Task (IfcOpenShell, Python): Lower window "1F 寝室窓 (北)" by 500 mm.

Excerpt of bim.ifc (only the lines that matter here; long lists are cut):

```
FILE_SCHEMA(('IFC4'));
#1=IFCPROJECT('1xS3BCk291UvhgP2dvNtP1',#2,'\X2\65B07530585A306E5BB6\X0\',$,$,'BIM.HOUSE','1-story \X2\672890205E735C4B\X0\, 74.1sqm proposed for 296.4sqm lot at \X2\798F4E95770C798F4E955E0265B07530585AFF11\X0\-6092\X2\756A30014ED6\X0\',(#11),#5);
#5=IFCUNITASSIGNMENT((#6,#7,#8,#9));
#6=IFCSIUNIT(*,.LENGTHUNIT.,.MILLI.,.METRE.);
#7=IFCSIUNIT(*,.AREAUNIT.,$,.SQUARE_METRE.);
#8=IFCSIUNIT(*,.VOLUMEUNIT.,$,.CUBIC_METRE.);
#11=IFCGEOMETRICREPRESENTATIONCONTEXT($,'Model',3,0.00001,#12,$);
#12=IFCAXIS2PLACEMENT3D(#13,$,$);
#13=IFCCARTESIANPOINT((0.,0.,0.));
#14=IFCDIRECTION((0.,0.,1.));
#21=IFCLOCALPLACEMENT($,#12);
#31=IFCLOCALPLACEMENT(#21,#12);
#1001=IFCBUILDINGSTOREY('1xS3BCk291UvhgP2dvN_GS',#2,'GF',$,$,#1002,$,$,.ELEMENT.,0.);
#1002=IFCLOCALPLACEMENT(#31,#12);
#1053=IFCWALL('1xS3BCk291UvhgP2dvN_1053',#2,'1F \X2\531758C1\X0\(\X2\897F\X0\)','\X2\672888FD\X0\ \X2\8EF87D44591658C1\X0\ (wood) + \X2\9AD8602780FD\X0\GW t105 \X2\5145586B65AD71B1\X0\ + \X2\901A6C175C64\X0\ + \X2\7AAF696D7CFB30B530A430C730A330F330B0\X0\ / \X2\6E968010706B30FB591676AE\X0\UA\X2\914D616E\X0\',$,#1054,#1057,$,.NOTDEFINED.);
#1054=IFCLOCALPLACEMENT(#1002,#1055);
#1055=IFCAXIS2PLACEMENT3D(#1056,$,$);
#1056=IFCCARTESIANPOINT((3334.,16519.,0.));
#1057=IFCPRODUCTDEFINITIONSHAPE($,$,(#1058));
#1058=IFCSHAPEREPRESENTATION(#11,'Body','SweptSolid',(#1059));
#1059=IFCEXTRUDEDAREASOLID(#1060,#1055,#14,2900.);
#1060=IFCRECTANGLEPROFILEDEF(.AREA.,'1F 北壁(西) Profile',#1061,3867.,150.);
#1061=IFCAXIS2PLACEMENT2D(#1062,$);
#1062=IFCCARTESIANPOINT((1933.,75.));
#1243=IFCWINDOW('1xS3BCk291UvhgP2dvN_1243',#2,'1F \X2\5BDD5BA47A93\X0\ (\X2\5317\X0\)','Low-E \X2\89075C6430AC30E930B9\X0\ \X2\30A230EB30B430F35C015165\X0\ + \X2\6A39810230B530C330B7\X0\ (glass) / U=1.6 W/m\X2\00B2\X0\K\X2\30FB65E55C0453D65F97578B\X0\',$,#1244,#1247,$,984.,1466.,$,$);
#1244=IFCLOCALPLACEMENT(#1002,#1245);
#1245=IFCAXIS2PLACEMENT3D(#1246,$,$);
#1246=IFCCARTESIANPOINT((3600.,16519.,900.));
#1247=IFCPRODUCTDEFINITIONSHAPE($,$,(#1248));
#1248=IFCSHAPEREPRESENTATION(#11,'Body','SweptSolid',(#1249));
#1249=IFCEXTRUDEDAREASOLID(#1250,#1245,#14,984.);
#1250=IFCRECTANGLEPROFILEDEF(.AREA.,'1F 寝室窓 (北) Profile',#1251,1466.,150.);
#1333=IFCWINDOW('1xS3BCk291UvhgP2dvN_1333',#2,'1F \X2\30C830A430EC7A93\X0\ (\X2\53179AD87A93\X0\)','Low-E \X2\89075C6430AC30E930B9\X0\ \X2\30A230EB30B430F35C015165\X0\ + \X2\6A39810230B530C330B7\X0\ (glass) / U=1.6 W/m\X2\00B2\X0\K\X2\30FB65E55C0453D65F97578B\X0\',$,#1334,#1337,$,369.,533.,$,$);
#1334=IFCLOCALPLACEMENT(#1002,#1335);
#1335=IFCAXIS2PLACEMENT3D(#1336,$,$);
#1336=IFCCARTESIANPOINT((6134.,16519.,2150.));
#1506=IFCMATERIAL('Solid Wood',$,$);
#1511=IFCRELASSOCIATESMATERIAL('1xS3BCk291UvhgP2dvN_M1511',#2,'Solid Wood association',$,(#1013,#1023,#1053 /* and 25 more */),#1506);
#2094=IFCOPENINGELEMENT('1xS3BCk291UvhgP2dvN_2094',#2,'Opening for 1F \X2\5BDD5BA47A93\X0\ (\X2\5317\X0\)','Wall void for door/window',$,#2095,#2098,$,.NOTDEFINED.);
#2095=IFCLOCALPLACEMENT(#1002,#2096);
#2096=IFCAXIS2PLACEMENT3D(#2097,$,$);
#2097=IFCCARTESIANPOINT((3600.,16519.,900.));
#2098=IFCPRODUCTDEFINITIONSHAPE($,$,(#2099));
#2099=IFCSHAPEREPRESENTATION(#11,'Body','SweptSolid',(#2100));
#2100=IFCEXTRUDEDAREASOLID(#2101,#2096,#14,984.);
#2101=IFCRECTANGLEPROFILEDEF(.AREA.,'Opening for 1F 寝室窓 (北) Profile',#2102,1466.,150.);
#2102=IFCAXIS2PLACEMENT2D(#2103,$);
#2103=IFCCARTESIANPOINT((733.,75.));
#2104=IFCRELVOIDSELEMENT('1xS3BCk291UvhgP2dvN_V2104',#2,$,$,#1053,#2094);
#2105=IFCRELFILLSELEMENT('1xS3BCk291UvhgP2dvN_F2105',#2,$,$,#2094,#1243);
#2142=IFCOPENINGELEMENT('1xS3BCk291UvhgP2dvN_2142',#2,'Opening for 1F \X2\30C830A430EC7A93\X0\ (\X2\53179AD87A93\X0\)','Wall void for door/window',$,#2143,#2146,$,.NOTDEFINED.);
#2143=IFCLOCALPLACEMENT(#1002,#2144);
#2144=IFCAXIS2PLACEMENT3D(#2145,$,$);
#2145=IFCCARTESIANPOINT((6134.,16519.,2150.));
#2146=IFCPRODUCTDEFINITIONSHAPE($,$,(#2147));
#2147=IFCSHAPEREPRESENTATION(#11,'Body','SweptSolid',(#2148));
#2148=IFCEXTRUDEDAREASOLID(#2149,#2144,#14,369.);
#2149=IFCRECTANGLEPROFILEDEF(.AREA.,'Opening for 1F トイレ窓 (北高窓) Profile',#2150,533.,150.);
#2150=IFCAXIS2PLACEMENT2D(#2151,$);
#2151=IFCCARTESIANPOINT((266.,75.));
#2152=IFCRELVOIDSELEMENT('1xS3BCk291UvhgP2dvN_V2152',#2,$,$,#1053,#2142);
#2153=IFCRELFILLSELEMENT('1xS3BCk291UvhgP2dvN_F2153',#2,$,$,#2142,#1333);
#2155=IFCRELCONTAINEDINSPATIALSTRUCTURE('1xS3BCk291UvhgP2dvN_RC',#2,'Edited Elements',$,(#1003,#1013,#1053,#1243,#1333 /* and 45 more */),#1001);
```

```python
import numpy as np
import ifcopenshell
import ifcopenshell.api.geometry
import ifcopenshell.util.placement
import ifcopenshell.util.unit

model = ifcopenshell.open("bim.ifc")
unit_scale = ifcopenshell.util.unit.calculate_unit_scale(model)

window = model.by_id(1243)
opening = window.FillsVoids[0].RelatingOpeningElement
dz = -0.5 / unit_scale

shift = np.array([0.0, 0.0, dz])
# The window is not placed relative to its opening, so move both.
for product in (opening, window):
    matrix = ifcopenshell.util.placement.get_local_placement(product.ObjectPlacement)
    matrix[:3, 3] += shift
    ifcopenshell.api.geometry.edit_object_placement(model, product=product, matrix=matrix, is_si=False)

print(f"moved by {dz * unit_scale:+.3f} m")

model.write("bim_v2.ifc")
```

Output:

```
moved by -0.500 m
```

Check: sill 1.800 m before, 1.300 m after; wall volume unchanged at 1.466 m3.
